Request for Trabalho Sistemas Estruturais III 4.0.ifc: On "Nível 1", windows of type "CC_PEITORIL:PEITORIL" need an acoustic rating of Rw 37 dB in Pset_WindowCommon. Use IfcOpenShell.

First a look at what the model holds.

```python
import ifcopenshell
import ifcopenshell.util.element

model = ifcopenshell.open("Trabalho Sistemas Estruturais III 4.0.ifc")
print(model.schema)
storey = next(s for s in model.by_type("IfcBuildingStorey") if s.Name == "Nível 1")
windows = [e for e in ifcopenshell.util.element.get_decomposition(storey) if e.is_a("IfcWindow")]
seen = {}
for e in windows:
    element_type = ifcopenshell.util.element.get_type(e)
    key = (element_type.Name if element_type != e and element_type else None, ifcopenshell.util.element.get_pset(e, "Pset_WindowCommon", "AcousticRating"))
    seen[key] = seen.get(key, 0) + 1
for (name, value), count in sorted(seen.items(), key=str):
    print(count, "x", name, "|", value)
```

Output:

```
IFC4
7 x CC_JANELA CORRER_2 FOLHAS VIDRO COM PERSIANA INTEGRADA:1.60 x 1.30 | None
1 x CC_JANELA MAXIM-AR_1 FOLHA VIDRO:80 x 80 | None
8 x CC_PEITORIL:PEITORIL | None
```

```python
import ifcopenshell
import ifcopenshell.api.pset
import ifcopenshell.util.element

model = ifcopenshell.open("Trabalho Sistemas Estruturais III 4.0.ifc")

storey = next(s for s in model.by_type("IfcBuildingStorey") if s.Name == "Nível 1")
windows = [e for e in ifcopenshell.util.element.get_decomposition(storey) if e.is_a("IfcWindow")]

count = 0
for e in windows:
    element_type = ifcopenshell.util.element.get_type(e)
    if element_type in (None, e) or element_type.Name != "CC_PEITORIL:PEITORIL":
        continue
    # add_pset returns the element's existing set when there is one.
    pset = ifcopenshell.api.pset.add_pset(model, product=e, name="Pset_WindowCommon")
    ifcopenshell.api.pset.edit_pset(model, pset=pset, properties={"AcousticRating": "Rw 37 dB"})
    count += 1

print(count, "windows updated")

model.write("Trabalho Sistemas Estruturais III 4.0-out.ifc")
```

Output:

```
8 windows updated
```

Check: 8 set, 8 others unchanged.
